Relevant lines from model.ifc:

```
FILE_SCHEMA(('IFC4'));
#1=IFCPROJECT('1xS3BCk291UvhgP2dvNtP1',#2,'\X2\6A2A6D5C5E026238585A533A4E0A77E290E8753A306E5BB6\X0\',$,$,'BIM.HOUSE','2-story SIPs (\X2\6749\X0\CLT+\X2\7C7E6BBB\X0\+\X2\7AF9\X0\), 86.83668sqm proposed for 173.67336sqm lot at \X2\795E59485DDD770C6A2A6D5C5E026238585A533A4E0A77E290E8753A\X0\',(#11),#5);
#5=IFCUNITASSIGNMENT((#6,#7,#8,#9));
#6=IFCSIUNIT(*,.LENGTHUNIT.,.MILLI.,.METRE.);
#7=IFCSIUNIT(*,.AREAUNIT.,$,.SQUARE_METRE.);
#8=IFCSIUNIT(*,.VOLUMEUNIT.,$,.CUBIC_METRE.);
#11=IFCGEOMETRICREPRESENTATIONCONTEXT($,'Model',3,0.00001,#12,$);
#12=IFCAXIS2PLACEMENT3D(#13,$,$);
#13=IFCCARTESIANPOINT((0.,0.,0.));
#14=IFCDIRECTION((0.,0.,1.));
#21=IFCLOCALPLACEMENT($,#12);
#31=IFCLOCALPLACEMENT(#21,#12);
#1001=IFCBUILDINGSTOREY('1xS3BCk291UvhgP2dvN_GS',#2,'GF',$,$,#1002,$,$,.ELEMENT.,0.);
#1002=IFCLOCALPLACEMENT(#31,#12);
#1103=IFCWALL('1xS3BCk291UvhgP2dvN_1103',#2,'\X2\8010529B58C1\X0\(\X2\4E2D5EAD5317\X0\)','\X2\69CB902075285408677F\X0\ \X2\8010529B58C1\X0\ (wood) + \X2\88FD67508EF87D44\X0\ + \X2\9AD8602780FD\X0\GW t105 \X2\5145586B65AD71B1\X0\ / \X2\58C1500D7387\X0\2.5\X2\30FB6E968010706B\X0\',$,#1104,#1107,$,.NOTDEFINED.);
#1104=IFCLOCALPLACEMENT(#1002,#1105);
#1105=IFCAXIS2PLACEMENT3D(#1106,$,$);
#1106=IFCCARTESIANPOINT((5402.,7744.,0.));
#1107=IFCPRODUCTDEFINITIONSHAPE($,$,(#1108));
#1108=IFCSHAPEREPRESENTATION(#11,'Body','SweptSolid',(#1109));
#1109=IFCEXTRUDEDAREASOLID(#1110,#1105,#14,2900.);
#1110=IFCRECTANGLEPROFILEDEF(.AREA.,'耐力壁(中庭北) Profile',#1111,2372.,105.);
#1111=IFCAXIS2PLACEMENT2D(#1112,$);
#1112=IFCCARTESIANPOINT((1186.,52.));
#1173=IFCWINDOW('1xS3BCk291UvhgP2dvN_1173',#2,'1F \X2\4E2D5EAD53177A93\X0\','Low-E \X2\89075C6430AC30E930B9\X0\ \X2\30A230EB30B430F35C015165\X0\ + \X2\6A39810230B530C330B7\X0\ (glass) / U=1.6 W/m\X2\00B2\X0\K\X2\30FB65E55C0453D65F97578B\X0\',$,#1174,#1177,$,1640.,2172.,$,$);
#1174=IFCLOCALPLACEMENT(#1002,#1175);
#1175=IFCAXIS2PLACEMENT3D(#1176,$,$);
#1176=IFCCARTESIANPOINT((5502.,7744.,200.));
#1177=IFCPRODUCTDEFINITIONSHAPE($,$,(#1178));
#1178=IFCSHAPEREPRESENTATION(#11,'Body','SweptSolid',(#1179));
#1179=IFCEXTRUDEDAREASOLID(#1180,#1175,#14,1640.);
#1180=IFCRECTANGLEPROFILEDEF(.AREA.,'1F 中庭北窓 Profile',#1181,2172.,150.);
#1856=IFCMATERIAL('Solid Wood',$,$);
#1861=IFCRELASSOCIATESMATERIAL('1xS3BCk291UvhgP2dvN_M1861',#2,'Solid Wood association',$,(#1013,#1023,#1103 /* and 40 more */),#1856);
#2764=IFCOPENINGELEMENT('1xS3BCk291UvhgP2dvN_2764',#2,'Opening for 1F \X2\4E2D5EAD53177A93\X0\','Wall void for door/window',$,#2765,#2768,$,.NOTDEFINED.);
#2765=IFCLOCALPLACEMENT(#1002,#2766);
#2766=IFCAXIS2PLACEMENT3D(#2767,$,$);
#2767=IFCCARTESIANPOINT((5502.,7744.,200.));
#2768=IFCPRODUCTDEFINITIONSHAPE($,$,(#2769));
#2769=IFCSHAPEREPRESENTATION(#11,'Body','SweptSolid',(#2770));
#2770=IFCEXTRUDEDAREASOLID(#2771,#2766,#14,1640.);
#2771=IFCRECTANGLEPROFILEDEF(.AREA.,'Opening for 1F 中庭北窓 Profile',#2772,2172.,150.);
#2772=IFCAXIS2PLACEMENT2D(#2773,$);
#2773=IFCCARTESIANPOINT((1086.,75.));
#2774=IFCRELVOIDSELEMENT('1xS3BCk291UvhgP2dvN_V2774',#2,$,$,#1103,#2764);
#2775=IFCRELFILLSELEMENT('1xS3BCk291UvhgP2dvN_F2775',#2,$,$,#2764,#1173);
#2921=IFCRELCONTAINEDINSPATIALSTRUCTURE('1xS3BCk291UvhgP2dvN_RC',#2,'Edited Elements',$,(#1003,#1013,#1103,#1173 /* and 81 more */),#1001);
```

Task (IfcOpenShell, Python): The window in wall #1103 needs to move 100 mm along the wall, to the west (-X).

```python
import ifcopenshell
import ifcopenshell.api.geometry
import ifcopenshell.util.placement
import ifcopenshell.util.unit

model = ifcopenshell.open("model.ifc")
unit_scale = ifcopenshell.util.unit.calculate_unit_scale(model)

window = model.by_guid("1xS3BCk291UvhgP2dvN_1173")
opening = window.FillsVoids[0].RelatingOpeningElement
wall = opening.VoidsElements[0].RelatingBuildingElement

wall_matrix = ifcopenshell.util.placement.get_local_placement(wall.ObjectPlacement)
shift = wall_matrix[:3, 0] * -0.1 / unit_scale
before = ifcopenshell.util.placement.get_local_placement(window.ObjectPlacement)[:3, 3].copy()

# The window is not placed relative to its opening, so move both.
for product in (opening, window):
    matrix = ifcopenshell.util.placement.get_local_placement(product.ObjectPlacement)
    matrix[:3, 3] += shift
    ifcopenshell.api.geometry.edit_object_placement(model, product=product, matrix=matrix, is_si=False)

after = ifcopenshell.util.placement.get_local_placement(window.ObjectPlacement)[:3, 3]
print("window moved by", (after - before).round(3) + 0.0)

model.write("model_updated.ifc")
```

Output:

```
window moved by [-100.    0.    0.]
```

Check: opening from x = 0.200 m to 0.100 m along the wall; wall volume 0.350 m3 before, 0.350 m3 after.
